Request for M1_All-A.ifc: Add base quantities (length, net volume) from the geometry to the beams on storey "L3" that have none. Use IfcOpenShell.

First a look at what the model holds.

```python
import ifcopenshell
import ifcopenshell.util.element
import ifcopenshell.util.unit

model = ifcopenshell.open("M1_All-A.ifc")
print(model.schema)
for unit_type in ("LENGTHUNIT", "AREAUNIT", "VOLUMEUNIT"):
    print(unit_type, ifcopenshell.util.unit.calculate_unit_scale(model, unit_type))
storey = next(s for s in model.by_type("IfcBuildingStorey") if s.Name == "L3")
beams = [e for e in ifcopenshell.util.element.get_decomposition(storey) if e.is_a("IfcBeam")]
for e in sorted(beams, key=lambda e: e.id()):
    print(e.id(), e.is_a(), e.Name, list(ifcopenshell.util.element.get_psets(e, qtos_only=True)), sep=" | ")
```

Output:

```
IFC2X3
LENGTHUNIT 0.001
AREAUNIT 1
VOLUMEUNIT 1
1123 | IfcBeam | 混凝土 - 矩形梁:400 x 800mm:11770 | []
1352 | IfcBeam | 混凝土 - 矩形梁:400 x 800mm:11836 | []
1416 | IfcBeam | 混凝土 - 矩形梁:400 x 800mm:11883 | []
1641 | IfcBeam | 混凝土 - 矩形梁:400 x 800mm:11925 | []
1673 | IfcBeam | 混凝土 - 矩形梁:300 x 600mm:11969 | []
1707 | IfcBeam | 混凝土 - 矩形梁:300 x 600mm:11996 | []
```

```python
import ifcopenshell
import ifcopenshell.api.pset
import ifcopenshell.geom
import ifcopenshell.util.element
import ifcopenshell.util.shape
import ifcopenshell.util.unit

model = ifcopenshell.open("M1_All-A.ifc")
unit_scale = ifcopenshell.util.unit.calculate_unit_scale(model)
volume_scale = ifcopenshell.util.unit.calculate_unit_scale(model, "VOLUMEUNIT")
settings = ifcopenshell.geom.settings()

storey = next(s for s in model.by_type("IfcBuildingStorey") if s.Name == "L3")
beams = [e for e in ifcopenshell.util.element.get_decomposition(storey) if e.is_a("IfcBeam")]

for e in sorted(beams, key=lambda e: e.id()):
    if ifcopenshell.util.element.get_psets(e, qtos_only=True, should_inherit=False):
        continue
    # Geometry comes back in metres, in the element's own axes.
    shape = ifcopenshell.geom.create_shape(settings, e)
    values = {
        "Length": ifcopenshell.util.shape.get_max_xyz(shape.geometry) / unit_scale,
        "NetVolume": ifcopenshell.util.shape.get_volume(shape.geometry) / volume_scale,
    }
    qto = ifcopenshell.api.pset.add_qto(model, product=e, name="BaseQuantities")
    ifcopenshell.api.pset.edit_qto(model, qto=qto, properties=values)
    print(e.id(), {k: round(v, 3) for k, v in values.items()})

model.write("M1_All-A_v2.ifc")
```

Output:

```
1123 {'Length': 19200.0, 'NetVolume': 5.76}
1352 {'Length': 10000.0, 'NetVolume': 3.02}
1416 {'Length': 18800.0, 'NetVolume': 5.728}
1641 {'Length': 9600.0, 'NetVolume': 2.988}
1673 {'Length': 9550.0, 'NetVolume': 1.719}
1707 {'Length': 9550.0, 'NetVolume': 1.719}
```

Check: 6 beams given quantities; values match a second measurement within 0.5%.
